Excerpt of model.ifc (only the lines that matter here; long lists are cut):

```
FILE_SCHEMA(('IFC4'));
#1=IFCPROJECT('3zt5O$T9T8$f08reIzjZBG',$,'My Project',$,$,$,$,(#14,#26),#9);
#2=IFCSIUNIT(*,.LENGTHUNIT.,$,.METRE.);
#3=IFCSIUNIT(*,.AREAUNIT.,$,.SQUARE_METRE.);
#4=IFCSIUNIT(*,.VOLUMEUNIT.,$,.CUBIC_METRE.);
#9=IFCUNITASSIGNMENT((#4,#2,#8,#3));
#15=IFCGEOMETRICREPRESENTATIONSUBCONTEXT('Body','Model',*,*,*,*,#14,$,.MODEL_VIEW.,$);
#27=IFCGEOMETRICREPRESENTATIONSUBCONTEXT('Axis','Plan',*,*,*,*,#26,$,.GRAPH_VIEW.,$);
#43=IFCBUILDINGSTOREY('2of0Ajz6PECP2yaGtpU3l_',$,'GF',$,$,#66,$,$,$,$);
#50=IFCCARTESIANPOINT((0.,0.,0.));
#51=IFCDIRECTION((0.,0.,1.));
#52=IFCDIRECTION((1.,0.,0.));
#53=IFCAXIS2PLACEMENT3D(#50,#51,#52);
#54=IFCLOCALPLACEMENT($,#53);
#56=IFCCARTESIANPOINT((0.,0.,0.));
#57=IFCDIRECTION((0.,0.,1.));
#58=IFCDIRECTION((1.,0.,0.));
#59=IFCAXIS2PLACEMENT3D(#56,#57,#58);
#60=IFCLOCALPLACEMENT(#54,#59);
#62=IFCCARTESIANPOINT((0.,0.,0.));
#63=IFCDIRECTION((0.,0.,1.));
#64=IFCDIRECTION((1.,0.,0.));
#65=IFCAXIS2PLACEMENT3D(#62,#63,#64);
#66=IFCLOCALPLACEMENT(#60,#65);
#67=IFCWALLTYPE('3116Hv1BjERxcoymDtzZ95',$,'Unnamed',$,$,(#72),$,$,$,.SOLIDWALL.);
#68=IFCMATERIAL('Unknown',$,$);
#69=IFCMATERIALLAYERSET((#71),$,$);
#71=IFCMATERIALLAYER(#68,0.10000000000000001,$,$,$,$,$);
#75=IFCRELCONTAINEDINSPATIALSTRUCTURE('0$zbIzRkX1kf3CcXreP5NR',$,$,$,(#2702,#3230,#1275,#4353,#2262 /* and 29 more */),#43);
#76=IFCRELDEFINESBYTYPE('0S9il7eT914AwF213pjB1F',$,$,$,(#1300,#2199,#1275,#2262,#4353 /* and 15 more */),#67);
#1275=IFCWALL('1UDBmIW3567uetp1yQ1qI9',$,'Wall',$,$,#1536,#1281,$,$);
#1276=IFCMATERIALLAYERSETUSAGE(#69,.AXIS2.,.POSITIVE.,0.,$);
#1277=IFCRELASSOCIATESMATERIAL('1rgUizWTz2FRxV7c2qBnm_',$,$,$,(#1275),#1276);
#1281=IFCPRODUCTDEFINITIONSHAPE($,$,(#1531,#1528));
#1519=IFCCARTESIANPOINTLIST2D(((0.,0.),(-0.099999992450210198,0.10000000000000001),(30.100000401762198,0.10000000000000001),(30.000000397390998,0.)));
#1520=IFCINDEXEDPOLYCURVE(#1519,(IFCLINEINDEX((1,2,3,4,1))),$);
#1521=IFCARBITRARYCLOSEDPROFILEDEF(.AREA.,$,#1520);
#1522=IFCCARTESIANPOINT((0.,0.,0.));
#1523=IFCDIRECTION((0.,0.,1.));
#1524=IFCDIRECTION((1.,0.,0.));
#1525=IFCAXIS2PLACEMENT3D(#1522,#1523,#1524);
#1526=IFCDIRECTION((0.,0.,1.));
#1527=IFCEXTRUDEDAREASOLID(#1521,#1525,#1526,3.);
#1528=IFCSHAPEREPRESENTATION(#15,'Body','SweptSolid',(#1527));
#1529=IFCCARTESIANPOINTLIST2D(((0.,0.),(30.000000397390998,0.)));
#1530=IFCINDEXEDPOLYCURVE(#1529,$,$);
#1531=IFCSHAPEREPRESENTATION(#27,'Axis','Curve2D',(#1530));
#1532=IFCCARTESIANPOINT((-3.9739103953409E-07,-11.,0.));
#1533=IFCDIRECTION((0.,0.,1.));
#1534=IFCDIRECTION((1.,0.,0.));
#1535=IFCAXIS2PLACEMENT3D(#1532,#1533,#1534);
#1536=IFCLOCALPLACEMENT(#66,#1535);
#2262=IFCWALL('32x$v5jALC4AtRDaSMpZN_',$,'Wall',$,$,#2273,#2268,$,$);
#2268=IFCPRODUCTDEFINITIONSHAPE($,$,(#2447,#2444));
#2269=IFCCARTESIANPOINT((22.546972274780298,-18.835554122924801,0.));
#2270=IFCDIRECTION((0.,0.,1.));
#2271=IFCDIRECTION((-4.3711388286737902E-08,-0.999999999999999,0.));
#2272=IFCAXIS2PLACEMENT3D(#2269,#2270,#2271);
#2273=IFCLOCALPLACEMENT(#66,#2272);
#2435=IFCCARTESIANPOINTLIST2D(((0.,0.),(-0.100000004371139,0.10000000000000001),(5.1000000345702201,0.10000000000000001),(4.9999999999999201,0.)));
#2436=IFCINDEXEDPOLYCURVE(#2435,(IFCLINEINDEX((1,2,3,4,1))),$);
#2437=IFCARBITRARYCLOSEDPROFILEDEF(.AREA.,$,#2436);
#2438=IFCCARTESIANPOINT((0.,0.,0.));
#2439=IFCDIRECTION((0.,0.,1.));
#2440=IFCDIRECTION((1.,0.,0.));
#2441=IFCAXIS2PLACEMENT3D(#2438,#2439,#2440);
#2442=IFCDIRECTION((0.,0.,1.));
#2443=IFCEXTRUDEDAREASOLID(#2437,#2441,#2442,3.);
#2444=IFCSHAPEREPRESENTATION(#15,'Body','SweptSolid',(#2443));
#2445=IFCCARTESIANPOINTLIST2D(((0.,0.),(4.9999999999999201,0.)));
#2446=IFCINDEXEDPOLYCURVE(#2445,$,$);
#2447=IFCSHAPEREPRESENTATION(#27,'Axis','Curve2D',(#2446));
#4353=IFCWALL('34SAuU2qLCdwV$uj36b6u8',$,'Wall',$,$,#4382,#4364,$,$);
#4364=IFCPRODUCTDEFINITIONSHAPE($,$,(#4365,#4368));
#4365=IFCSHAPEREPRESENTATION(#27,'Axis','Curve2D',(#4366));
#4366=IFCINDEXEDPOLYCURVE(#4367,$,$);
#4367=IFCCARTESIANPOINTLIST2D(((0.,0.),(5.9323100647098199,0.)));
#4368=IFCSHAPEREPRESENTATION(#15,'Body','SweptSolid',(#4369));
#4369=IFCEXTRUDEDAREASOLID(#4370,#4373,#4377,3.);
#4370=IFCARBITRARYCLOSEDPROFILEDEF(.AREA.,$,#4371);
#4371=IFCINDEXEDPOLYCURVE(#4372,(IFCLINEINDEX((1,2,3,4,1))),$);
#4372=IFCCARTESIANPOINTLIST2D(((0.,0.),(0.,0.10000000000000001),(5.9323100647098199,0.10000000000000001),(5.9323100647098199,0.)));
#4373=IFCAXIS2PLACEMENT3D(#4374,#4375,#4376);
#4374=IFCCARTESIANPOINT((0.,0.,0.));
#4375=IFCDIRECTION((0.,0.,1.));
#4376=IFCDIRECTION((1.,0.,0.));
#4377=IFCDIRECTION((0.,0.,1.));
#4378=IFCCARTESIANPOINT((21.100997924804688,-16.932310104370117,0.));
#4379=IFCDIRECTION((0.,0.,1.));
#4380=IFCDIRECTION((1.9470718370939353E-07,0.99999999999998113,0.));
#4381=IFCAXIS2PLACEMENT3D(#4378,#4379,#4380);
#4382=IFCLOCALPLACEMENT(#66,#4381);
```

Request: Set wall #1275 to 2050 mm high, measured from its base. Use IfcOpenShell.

```python
import ifcopenshell
import ifcopenshell.geom
import ifcopenshell.util.representation
import ifcopenshell.util.shape
import ifcopenshell.util.unit

model = ifcopenshell.open("model.ifc")
unit_scale = ifcopenshell.util.unit.calculate_unit_scale(model)
settings = ifcopenshell.geom.settings()


def volume(element):
    """Net volume in cubic metres, openings subtracted."""
    shape = ifcopenshell.geom.create_shape(settings, element)
    return ifcopenshell.util.shape.get_volume(shape.geometry)


wall = model.by_guid("1UDBmIW3567uetp1yQ1qI9")
before = volume(wall)

body = ifcopenshell.util.representation.get_representation(wall, "Model", "Body")
solid = body.Items[0]
old_height = solid.Depth
solid.Depth = 2.05 / unit_scale
after = volume(wall)

print(f"height {old_height:g} -> {solid.Depth:g}, volume {before:.3f} -> {after:.3f} m3")

model.write("model_edited.ifc")
```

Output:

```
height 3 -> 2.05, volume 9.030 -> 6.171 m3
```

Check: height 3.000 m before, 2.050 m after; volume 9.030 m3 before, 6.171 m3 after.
